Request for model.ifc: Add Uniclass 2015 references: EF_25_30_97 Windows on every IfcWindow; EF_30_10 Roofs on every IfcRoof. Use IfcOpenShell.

First a look at what the model holds.

```python
import ifcopenshell

model = ifcopenshell.open("model.ifc")
print(model.schema)
print("classifications:", [c.Name for c in model.by_type("IfcClassification")])
for ifc_class in ("IfcDoor", "IfcRoof", "IfcStair", "IfcWall", "IfcWindow"):
    print(ifc_class, len(model.by_type(ifc_class)))
```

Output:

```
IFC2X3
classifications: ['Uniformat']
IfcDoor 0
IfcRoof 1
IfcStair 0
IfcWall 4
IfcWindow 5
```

```python
import ifcopenshell
import ifcopenshell.api.classification

model = ifcopenshell.open("model.ifc")

# IFC2X3 requires Source and Edition and has no link from the project to the system.
system = model.create_entity("IfcClassification", Source="NBS", Edition="2015", Name="Uniclass 2015")

codes = {
    "IfcWindow": ("EF_25_30_97", "Windows"),
    "IfcRoof": ("EF_30_10", "Roofs"),
}
for ifc_class, (code, name) in codes.items():
    products = model.by_type(ifc_class)
    ifcopenshell.api.classification.add_reference(
        model, products=products, classification=system, identification=code, name=name
    )
    print(code, len(products))

model.write("model_v2.ifc")
```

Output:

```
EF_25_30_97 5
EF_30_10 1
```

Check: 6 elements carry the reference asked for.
